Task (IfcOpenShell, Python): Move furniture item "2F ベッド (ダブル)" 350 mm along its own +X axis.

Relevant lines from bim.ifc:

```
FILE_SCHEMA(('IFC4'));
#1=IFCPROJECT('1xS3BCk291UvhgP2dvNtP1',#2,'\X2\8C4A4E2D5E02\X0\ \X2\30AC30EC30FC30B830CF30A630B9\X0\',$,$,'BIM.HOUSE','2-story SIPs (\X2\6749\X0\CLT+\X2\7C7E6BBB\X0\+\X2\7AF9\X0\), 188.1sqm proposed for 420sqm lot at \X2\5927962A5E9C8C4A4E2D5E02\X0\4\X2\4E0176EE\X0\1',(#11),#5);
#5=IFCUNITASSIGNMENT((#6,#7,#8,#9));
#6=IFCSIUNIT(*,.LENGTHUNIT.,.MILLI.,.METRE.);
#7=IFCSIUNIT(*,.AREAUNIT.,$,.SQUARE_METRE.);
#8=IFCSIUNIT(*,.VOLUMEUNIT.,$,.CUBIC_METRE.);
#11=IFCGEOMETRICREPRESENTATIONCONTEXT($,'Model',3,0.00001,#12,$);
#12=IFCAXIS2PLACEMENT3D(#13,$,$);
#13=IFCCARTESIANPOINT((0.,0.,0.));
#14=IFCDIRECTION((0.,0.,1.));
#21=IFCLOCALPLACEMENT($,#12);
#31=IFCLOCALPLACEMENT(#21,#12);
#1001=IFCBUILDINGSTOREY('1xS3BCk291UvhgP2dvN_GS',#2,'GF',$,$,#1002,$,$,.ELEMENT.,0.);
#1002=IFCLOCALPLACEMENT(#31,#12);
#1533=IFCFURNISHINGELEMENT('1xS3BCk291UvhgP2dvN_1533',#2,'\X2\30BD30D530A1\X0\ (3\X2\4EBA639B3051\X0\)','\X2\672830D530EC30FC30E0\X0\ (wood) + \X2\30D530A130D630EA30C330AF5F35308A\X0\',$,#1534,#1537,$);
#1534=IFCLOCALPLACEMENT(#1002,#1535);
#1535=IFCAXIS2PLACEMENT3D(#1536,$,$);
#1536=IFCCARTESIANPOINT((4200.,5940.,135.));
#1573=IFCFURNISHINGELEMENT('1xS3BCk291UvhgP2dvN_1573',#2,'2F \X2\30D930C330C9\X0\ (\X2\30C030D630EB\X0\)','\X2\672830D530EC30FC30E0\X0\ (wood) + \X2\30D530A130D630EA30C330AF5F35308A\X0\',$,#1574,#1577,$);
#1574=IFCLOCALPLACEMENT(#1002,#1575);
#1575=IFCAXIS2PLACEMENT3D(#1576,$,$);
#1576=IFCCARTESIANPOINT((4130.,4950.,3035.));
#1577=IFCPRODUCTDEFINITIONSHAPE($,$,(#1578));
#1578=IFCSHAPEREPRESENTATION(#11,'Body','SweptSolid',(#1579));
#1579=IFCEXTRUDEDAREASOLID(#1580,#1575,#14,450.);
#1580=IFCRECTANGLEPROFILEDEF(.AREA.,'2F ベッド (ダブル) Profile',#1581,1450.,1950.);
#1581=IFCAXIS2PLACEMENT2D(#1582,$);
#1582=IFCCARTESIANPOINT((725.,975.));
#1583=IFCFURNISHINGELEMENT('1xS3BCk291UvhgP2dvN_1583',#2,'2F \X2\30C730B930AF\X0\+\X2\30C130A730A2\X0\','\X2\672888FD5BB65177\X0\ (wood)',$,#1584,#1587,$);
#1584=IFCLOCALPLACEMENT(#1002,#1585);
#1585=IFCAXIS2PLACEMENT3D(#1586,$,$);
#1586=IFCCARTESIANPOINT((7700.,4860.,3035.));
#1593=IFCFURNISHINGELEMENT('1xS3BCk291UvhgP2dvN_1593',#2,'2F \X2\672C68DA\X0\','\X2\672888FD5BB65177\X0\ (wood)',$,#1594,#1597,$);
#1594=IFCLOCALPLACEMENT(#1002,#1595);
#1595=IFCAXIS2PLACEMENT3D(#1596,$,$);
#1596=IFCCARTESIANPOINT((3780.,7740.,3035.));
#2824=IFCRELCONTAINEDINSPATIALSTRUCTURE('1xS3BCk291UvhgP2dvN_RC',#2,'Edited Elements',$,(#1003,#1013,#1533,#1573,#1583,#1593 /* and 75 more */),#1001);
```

```python
import ifcopenshell
import ifcopenshell.api.geometry
import ifcopenshell.util.placement
import ifcopenshell.util.unit

model = ifcopenshell.open("bim.ifc")
unit_scale = ifcopenshell.util.unit.calculate_unit_scale(model)

item = model.by_guid("1xS3BCk291UvhgP2dvN_1573")
matrix = ifcopenshell.util.placement.get_local_placement(item.ObjectPlacement)
matrix[:3, 3] += matrix[:3, 0] * 0.35 / unit_scale
ifcopenshell.api.geometry.edit_object_placement(model, product=item, matrix=matrix, is_si=False)

print(ifcopenshell.util.placement.get_local_placement(item.ObjectPlacement).round(3) + 0.0)

model.write("bim_rev.ifc")
```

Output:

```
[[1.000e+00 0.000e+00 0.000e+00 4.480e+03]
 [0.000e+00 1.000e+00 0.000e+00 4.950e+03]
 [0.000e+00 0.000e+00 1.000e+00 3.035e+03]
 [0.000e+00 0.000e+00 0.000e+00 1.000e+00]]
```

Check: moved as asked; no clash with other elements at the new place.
